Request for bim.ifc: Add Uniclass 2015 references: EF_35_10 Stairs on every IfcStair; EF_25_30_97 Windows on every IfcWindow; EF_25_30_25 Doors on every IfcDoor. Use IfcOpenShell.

First a look at what the model holds.

```python
import ifcopenshell

model = ifcopenshell.open("bim.ifc")
print(model.schema)
print("classifications:", [c.Name for c in model.by_type("IfcClassification")])
for ifc_class in ("IfcDoor", "IfcRoof", "IfcStair", "IfcWall", "IfcWindow"):
    print(ifc_class, len(model.by_type(ifc_class)))
```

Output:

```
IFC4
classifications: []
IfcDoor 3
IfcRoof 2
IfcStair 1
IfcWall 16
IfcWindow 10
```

```python
import ifcopenshell
import ifcopenshell.api.classification

model = ifcopenshell.open("bim.ifc")

system = ifcopenshell.api.classification.add_classification(model, classification="Uniclass 2015")

codes = {
    "IfcStair": ("EF_35_10", "Stairs"),
    "IfcWindow": ("EF_25_30_97", "Windows"),
    "IfcDoor": ("EF_25_30_25", "Doors"),
}
for ifc_class, (code, name) in codes.items():
    products = model.by_type(ifc_class)
    ifcopenshell.api.classification.add_reference(
        model, products=products, classification=system, identification=code, name=name
    )
    print(code, len(products))

model.write("bim_updated.ifc")
```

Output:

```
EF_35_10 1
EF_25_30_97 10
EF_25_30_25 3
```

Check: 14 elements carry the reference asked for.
